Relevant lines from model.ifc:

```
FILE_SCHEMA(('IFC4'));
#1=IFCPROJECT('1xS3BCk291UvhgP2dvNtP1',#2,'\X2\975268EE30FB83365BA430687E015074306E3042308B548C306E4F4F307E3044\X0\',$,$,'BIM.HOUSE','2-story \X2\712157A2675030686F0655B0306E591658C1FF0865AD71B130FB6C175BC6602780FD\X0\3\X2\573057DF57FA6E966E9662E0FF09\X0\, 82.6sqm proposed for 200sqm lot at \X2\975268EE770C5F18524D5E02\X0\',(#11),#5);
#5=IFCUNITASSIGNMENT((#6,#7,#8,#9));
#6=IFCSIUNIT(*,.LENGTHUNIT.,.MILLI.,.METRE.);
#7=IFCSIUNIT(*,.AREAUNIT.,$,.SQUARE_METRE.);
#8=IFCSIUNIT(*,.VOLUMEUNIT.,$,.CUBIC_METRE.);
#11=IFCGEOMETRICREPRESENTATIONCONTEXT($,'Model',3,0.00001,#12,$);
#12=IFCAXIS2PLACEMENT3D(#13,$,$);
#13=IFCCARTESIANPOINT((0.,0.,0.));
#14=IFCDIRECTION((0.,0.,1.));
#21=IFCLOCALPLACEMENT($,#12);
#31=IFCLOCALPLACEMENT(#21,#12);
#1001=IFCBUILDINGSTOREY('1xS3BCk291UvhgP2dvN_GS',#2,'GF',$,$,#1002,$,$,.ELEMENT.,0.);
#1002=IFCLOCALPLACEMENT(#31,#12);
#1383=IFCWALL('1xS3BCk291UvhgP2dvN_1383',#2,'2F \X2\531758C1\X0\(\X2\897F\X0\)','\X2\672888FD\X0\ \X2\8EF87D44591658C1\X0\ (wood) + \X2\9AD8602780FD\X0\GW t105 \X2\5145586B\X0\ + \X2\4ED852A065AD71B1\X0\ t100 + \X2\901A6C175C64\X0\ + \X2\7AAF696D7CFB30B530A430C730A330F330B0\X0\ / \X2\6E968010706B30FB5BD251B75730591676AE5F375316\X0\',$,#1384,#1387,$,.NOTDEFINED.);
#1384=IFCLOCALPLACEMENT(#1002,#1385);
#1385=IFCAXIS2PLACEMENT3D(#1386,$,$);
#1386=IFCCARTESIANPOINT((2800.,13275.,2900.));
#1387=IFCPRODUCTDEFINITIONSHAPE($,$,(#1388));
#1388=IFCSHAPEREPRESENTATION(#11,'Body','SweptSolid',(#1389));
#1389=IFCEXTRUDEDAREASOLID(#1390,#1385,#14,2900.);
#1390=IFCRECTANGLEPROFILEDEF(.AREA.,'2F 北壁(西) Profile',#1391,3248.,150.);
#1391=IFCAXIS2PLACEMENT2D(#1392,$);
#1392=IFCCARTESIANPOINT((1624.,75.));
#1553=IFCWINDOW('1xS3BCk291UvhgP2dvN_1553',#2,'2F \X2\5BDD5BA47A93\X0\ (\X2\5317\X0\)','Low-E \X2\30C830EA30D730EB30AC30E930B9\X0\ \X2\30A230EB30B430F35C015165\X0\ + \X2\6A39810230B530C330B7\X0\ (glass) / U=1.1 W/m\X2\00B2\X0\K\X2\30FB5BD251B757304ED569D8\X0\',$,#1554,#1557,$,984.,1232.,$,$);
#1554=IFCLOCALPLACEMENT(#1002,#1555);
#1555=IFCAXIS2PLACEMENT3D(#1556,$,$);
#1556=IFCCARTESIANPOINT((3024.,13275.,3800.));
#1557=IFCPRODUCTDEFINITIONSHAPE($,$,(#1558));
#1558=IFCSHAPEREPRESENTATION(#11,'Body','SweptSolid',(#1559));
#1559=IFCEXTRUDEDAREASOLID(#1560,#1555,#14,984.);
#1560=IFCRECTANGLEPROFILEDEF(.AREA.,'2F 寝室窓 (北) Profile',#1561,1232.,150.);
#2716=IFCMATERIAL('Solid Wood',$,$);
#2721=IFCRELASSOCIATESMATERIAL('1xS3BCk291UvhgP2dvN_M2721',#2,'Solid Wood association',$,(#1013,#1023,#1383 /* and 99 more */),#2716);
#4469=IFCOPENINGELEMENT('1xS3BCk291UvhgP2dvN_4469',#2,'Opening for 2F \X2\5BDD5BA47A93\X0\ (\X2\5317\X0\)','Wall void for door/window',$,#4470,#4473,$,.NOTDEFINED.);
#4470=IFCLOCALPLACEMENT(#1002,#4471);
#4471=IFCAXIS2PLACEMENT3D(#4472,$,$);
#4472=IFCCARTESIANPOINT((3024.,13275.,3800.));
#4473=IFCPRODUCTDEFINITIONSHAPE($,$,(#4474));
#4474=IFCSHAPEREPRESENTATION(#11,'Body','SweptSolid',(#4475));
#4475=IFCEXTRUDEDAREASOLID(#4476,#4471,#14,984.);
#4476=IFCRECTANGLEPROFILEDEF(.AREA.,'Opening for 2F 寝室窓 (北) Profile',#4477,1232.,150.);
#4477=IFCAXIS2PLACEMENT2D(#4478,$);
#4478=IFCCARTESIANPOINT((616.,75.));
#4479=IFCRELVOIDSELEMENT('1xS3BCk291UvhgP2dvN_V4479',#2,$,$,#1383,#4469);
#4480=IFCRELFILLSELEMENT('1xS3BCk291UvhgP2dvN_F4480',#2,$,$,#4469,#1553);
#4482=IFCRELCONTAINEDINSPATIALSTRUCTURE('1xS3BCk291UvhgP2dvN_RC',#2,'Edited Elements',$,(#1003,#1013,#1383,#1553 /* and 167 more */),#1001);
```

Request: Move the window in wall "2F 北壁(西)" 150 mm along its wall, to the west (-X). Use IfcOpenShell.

```python
import ifcopenshell
import ifcopenshell.api.geometry
import ifcopenshell.util.placement

model = ifcopenshell.open("model.ifc")

window = model.by_guid("1xS3BCk291UvhgP2dvN_1553")
opening = window.FillsVoids[0].RelatingOpeningElement
wall = opening.VoidsElements[0].RelatingBuildingElement

wall_matrix = ifcopenshell.util.placement.get_local_placement(wall.ObjectPlacement)
shift = wall_matrix[:3, 0] * -150.0
before = ifcopenshell.util.placement.get_local_placement(window.ObjectPlacement)[:3, 3].copy()

# The window is not placed relative to its opening, so move both.
for product in (opening, window):
    matrix = ifcopenshell.util.placement.get_local_placement(product.ObjectPlacement)
    matrix[:3, 3] += shift
    ifcopenshell.api.geometry.edit_object_placement(model, product=product, matrix=matrix, is_si=False)

after = ifcopenshell.util.placement.get_local_placement(window.ObjectPlacement)[:3, 3]
print("window moved by", (after - before).round(3) + 0.0)

model.write("model_rev.ifc")
```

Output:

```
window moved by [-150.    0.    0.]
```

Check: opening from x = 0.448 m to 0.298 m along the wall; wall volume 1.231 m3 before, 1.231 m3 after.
